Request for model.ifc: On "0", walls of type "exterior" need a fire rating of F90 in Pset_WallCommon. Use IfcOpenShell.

First a look at what the model holds.

```python
import ifcopenshell
import ifcopenshell.util.element

model = ifcopenshell.open("model.ifc")
print(model.schema)
storey = next(s for s in model.by_type("IfcBuildingStorey") if s.Name == "0")
walls = [e for e in ifcopenshell.util.element.get_decomposition(storey) if e.is_a("IfcWall")]
seen = {}
for e in walls:
    element_type = ifcopenshell.util.element.get_type(e)
    key = (element_type.Name if element_type != e and element_type else None, ifcopenshell.util.element.get_pset(e, "Pset_WallCommon", "FireRating"))
    seen[key] = seen.get(key, 0) + 1
for (name, value), count in sorted(seen.items(), key=str):
    print(count, "x", name, "|", value)
```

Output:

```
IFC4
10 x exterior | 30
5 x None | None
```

```python
import ifcopenshell
import ifcopenshell.api.pset
import ifcopenshell.util.element

model = ifcopenshell.open("model.ifc")

storey = next(s for s in model.by_type("IfcBuildingStorey") if s.Name == "0")
walls = [e for e in ifcopenshell.util.element.get_decomposition(storey) if e.is_a("IfcWall")]

count = 0
for e in walls:
    element_type = ifcopenshell.util.element.get_type(e)
    if element_type in (None, e) or element_type.Name != "exterior":
        continue
    # add_pset returns the element's existing set when there is one.
    pset = ifcopenshell.api.pset.add_pset(model, product=e, name="Pset_WallCommon")
    ifcopenshell.api.pset.edit_pset(model, pset=pset, properties={"FireRating": "F90"})
    count += 1

print(count, "walls updated")

model.write("model_rev.ifc")
```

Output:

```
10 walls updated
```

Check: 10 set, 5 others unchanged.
